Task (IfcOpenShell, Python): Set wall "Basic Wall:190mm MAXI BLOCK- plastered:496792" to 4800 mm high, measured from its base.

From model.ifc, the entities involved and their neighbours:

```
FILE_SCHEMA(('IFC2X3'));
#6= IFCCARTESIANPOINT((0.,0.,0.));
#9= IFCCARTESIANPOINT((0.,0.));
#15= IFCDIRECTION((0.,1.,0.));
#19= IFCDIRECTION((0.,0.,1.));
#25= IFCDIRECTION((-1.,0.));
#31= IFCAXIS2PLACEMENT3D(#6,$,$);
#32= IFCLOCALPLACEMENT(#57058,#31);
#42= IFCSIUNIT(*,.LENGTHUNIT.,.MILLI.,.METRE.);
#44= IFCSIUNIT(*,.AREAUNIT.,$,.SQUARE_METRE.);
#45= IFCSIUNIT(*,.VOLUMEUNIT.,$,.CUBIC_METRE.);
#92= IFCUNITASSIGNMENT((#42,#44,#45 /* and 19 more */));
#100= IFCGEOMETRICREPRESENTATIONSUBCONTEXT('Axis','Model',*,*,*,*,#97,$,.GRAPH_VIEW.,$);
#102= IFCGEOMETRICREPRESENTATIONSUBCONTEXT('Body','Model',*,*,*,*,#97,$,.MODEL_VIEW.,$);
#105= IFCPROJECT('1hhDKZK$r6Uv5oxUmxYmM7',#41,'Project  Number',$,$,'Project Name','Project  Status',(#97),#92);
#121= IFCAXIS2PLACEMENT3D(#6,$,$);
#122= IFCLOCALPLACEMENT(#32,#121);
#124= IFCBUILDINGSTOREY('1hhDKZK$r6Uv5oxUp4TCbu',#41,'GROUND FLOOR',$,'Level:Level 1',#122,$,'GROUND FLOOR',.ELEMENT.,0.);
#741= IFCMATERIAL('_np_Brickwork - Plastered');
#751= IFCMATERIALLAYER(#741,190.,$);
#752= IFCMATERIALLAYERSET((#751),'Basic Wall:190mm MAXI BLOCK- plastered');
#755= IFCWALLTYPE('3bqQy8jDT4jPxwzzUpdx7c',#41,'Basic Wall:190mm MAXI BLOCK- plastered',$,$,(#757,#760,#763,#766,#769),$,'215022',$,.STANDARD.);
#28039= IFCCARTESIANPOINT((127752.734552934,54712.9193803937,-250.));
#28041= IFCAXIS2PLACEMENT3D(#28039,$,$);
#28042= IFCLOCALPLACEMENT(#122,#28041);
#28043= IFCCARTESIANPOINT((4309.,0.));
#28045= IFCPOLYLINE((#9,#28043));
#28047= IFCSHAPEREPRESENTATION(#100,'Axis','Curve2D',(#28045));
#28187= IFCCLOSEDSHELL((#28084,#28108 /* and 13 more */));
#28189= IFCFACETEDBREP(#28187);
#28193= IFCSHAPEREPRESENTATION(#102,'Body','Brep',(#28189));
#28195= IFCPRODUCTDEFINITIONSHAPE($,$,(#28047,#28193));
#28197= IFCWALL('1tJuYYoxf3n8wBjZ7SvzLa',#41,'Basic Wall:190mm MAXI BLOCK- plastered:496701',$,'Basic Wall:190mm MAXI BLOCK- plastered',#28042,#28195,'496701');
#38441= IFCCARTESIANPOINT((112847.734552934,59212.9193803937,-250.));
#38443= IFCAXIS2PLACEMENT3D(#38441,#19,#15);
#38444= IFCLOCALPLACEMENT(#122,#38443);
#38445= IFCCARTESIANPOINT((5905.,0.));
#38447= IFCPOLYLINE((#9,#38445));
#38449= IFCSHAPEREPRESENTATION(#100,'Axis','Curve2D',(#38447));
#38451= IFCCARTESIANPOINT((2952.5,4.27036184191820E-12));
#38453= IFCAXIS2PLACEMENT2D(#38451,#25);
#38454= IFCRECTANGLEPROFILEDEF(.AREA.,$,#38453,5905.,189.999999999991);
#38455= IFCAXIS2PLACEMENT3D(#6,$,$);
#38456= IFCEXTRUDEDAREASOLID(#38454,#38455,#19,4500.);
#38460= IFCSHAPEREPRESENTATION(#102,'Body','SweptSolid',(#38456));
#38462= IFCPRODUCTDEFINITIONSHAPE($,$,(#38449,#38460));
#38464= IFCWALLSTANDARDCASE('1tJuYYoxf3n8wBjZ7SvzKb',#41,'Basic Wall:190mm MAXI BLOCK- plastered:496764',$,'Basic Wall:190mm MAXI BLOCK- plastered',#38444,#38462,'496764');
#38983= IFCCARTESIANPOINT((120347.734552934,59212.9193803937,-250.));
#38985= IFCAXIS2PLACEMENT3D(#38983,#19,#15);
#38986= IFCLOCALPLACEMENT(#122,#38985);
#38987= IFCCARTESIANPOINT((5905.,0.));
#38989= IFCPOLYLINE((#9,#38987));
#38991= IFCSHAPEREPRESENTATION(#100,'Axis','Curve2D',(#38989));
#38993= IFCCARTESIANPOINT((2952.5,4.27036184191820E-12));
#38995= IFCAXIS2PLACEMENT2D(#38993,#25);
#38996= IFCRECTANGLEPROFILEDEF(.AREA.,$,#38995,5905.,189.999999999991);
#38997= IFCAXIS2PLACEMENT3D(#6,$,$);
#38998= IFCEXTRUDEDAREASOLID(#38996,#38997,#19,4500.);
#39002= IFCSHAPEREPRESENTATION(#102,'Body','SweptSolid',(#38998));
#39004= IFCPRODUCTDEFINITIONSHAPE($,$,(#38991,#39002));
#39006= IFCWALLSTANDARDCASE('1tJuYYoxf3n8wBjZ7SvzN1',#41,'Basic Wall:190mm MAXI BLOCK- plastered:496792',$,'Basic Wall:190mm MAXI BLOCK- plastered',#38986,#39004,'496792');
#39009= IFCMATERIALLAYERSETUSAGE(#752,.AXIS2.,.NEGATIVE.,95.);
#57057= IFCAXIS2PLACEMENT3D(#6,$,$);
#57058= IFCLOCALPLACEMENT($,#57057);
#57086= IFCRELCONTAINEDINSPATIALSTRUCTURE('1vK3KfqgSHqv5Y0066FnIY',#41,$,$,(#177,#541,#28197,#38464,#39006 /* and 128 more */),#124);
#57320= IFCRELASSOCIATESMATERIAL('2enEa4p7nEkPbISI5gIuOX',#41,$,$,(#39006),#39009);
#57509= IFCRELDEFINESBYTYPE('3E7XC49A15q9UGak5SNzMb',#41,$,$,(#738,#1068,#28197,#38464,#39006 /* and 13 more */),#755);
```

```python
import ifcopenshell
import ifcopenshell.geom
import ifcopenshell.util.representation
import ifcopenshell.util.shape

model = ifcopenshell.open("model.ifc")
settings = ifcopenshell.geom.settings()


def volume(element):
    """Net volume in cubic metres, openings subtracted."""
    shape = ifcopenshell.geom.create_shape(settings, element)
    return ifcopenshell.util.shape.get_volume(shape.geometry)


wall = model.by_guid("1tJuYYoxf3n8wBjZ7SvzN1")
before = volume(wall)

body = ifcopenshell.util.representation.get_representation(wall, "Model", "Body")
solid = body.Items[0]
old_height = solid.Depth
solid.Depth = 4800.0
after = volume(wall)

print(f"height {old_height:g} -> {solid.Depth:g}, volume {before:.3f} -> {after:.3f} m3")

model.write("model_rev.ifc")
```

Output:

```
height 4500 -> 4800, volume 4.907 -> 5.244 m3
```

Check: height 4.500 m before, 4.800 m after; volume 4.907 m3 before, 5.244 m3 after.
